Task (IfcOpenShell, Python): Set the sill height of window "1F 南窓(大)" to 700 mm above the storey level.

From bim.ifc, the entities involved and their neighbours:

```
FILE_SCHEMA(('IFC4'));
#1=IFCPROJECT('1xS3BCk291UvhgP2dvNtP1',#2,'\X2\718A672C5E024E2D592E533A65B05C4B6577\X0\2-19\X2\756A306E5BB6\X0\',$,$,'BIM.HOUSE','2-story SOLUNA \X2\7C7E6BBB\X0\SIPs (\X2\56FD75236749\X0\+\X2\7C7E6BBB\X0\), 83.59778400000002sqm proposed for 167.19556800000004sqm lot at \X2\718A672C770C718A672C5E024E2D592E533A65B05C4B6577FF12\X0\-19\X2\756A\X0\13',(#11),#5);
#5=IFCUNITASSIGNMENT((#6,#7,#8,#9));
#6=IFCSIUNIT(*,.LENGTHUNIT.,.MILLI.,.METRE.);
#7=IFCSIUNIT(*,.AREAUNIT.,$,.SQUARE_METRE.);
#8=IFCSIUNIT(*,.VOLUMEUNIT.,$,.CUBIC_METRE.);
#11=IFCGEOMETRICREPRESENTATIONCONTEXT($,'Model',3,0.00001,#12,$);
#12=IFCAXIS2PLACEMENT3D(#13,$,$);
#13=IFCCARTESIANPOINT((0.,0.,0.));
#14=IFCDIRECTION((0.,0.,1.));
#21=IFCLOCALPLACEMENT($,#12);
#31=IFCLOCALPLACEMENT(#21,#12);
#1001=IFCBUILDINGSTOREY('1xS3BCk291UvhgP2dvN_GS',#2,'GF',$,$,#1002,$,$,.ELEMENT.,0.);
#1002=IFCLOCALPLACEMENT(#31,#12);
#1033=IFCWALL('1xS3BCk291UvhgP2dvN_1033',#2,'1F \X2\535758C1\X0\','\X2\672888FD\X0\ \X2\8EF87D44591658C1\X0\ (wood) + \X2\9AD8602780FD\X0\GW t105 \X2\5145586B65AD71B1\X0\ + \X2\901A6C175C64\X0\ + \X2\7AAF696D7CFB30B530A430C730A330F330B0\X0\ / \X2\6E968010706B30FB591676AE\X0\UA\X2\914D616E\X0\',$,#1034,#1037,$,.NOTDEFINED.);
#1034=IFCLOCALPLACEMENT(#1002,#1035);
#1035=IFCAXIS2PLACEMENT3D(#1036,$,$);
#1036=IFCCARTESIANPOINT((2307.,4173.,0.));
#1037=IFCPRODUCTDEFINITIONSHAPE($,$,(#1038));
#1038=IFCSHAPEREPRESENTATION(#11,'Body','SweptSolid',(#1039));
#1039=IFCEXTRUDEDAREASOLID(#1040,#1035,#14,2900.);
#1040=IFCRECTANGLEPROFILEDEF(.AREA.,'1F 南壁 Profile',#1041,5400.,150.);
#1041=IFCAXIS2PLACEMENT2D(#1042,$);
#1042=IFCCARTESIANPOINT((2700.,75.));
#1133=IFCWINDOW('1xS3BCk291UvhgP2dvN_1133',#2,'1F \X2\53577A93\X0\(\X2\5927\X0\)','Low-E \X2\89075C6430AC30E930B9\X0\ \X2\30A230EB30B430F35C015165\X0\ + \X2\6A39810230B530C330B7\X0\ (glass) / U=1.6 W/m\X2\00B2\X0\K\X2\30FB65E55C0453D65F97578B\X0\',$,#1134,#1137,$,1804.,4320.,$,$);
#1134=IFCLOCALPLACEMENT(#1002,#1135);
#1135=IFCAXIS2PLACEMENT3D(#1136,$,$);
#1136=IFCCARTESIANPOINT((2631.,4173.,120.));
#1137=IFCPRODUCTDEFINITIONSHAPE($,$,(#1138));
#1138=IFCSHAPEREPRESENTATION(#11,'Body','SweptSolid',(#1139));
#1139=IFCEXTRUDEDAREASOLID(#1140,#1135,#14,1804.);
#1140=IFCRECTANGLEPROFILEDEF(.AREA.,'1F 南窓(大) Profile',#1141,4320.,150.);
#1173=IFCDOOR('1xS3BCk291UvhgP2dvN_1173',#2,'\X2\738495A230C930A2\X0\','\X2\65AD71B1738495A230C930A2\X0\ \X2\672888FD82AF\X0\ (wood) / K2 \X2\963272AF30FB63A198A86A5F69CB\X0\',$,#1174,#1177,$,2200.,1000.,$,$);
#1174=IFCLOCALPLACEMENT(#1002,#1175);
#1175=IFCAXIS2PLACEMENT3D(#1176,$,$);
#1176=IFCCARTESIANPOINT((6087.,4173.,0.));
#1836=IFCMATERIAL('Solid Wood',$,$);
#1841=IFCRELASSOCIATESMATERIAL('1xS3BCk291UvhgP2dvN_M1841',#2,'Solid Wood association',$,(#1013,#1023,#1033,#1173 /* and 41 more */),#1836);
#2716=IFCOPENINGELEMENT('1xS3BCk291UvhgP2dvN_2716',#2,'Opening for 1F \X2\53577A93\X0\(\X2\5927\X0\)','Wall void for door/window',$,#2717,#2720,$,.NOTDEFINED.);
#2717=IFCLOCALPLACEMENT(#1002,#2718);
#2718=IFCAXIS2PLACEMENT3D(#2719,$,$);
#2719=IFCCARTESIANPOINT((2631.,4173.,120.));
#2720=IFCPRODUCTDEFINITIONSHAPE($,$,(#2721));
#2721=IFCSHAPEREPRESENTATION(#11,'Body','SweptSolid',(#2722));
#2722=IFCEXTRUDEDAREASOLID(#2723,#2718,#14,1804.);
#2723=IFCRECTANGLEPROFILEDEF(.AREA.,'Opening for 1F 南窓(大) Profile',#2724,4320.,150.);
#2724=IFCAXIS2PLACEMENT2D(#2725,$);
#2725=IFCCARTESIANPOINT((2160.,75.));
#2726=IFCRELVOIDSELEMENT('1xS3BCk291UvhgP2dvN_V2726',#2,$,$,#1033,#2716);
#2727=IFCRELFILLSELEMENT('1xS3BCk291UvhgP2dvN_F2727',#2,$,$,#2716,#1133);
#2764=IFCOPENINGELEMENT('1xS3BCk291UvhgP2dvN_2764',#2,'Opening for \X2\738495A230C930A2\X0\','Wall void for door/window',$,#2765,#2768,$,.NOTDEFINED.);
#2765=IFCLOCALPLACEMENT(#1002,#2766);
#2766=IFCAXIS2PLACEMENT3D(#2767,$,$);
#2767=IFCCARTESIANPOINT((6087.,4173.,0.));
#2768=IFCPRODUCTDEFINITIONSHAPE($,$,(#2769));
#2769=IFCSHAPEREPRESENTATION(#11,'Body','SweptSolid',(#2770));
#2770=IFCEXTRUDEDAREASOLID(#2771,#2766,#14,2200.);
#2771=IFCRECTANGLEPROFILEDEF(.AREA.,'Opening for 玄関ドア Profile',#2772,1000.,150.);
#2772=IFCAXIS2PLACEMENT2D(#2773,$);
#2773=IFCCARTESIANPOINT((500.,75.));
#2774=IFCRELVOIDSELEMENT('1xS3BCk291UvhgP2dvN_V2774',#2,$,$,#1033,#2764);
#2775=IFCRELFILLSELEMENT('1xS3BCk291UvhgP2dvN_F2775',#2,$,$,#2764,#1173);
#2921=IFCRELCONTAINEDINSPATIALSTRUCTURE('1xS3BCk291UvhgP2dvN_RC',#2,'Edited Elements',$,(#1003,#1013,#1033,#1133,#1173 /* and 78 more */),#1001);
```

```python
import numpy as np
import ifcopenshell
import ifcopenshell.api.geometry
import ifcopenshell.geom
import ifcopenshell.util.element
import ifcopenshell.util.placement
import ifcopenshell.util.shape
import ifcopenshell.util.unit

model = ifcopenshell.open("bim.ifc")
unit_scale = ifcopenshell.util.unit.calculate_unit_scale(model)

window = model.by_guid("1xS3BCk291UvhgP2dvN_1133")
opening = window.FillsVoids[0].RelatingOpeningElement
storey = ifcopenshell.util.element.get_container(window, ifc_class="IfcBuildingStorey")
level = ifcopenshell.util.placement.get_local_placement(storey.ObjectPlacement)[2, 3]

# The opening's origin need not be at the sill, so measure its lowest point.
shape = ifcopenshell.geom.create_shape(ifcopenshell.geom.settings(), opening)
bottom = ifcopenshell.util.shape.get_shape_bottom_elevation(shape, shape.geometry) / unit_scale
dz = level + 0.7 / unit_scale - bottom

shift = np.array([0.0, 0.0, dz])
# The window is not placed relative to its opening, so move both.
for product in (opening, window):
    matrix = ifcopenshell.util.placement.get_local_placement(product.ObjectPlacement)
    matrix[:3, 3] += shift
    ifcopenshell.api.geometry.edit_object_placement(model, product=product, matrix=matrix, is_si=False)

print(f"moved by {dz * unit_scale:+.3f} m")

model.write("bim_rev.ifc")
```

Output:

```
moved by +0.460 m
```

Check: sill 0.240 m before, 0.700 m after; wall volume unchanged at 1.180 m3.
